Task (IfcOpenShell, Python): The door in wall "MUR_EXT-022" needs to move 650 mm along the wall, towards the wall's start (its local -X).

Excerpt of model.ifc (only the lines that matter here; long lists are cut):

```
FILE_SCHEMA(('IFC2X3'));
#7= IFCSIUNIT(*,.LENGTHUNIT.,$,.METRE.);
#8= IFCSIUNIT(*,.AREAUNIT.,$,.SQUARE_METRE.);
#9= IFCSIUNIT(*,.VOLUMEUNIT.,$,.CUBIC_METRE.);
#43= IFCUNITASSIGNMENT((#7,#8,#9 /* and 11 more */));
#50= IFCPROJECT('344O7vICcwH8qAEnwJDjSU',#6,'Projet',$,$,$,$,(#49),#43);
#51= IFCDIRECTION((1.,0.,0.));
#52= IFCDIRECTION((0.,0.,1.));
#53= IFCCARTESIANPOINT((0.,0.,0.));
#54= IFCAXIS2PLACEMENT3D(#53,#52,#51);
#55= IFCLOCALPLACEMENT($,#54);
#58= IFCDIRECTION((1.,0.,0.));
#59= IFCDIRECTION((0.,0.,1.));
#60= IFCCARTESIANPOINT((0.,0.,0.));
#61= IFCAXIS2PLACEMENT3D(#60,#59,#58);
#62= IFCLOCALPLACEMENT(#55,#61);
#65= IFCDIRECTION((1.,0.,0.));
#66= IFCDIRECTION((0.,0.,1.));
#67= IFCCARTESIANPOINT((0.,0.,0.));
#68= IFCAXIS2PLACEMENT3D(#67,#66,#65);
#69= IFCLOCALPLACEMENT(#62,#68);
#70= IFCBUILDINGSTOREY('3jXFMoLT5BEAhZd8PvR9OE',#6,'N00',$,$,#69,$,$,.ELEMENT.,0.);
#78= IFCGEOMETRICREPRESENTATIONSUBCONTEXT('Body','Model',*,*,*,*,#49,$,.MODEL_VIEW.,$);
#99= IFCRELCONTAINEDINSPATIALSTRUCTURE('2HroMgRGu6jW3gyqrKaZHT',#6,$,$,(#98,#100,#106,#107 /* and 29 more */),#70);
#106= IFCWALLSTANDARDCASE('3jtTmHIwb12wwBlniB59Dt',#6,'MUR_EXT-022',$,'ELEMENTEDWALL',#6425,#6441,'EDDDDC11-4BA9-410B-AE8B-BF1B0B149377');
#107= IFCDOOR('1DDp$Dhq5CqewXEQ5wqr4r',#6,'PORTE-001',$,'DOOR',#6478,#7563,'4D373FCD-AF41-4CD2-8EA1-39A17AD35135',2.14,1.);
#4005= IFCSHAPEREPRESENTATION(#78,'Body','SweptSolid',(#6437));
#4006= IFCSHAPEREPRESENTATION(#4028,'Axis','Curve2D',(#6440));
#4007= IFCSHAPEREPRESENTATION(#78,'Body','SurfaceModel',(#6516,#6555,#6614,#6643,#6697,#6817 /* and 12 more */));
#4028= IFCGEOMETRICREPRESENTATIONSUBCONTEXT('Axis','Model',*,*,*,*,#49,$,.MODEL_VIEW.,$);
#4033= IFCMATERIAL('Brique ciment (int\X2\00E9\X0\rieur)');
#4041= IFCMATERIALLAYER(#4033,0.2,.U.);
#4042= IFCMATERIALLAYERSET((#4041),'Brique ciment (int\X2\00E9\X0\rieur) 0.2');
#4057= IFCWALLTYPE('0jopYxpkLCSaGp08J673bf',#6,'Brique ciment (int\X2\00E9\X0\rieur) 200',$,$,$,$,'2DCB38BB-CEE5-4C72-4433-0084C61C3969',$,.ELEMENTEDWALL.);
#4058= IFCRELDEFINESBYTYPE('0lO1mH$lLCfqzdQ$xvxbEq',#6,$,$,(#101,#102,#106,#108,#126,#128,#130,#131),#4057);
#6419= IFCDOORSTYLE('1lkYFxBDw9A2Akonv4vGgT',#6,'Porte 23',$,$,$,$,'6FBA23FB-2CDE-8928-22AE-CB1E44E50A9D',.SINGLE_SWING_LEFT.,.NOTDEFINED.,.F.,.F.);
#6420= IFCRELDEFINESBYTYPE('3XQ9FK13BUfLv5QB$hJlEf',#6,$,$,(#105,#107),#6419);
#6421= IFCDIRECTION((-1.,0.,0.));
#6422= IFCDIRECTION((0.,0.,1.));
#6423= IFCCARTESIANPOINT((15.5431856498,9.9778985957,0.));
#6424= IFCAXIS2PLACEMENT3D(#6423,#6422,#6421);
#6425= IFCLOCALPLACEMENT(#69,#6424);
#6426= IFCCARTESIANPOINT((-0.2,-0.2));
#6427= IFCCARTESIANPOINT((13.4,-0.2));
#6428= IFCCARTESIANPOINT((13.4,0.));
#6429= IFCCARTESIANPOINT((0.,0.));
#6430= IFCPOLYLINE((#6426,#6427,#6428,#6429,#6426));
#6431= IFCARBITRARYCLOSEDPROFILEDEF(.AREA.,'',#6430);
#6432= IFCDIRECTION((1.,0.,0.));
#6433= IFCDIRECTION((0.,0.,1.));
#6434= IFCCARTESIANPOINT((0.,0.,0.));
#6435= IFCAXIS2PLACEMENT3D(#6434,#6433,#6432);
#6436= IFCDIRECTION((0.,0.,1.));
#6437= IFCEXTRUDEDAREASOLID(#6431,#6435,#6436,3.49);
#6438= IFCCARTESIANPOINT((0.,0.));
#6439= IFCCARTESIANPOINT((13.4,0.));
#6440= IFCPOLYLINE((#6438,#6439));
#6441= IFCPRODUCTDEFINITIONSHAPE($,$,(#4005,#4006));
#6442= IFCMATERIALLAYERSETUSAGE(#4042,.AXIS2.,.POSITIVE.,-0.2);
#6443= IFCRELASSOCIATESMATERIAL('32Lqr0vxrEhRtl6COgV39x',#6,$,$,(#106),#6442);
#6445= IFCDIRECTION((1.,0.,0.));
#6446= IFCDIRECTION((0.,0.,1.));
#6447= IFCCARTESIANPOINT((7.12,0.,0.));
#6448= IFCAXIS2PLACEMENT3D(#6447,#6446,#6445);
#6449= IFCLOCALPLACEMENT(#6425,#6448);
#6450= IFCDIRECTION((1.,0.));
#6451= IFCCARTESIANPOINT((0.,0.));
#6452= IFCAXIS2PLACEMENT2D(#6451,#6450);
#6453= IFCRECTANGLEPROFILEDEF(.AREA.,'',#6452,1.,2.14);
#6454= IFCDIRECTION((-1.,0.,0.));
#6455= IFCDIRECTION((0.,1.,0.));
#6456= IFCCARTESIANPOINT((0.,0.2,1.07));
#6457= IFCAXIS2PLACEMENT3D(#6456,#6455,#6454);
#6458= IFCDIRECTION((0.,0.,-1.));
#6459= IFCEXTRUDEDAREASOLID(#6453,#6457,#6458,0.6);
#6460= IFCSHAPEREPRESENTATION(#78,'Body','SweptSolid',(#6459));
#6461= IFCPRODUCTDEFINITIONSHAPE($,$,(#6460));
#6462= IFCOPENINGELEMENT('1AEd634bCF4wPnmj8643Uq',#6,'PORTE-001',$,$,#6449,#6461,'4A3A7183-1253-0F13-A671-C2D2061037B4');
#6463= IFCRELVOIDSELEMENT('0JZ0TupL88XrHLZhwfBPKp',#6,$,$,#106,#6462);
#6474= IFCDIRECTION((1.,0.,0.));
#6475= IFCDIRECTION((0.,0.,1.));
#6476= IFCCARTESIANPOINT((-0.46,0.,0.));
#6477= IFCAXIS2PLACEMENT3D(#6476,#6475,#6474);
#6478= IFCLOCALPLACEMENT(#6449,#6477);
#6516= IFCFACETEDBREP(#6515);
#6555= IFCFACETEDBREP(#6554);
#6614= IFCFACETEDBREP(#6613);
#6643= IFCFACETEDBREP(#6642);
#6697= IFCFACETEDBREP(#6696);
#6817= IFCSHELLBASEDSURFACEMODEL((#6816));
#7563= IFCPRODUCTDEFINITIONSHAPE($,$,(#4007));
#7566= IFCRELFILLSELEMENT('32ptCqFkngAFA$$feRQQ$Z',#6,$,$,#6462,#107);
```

```python
import ifcopenshell
import ifcopenshell.api.geometry
import ifcopenshell.util.placement
import ifcopenshell.util.unit

model = ifcopenshell.open("model.ifc")
unit_scale = ifcopenshell.util.unit.calculate_unit_scale(model)

door = model.by_id(107)
opening = door.FillsVoids[0].RelatingOpeningElement
wall = opening.VoidsElements[0].RelatingBuildingElement

wall_matrix = ifcopenshell.util.placement.get_local_placement(wall.ObjectPlacement)
shift = wall_matrix[:3, 0] * -0.65 / unit_scale
before = ifcopenshell.util.placement.get_local_placement(door.ObjectPlacement)[:3, 3].copy()

# The door is placed relative to its opening, so it follows when the opening moves.
matrix = ifcopenshell.util.placement.get_local_placement(opening.ObjectPlacement)
matrix[:3, 3] += shift
ifcopenshell.api.geometry.edit_object_placement(
    model, product=opening, matrix=matrix, is_si=False, should_transform_children=True
)

after = ifcopenshell.util.placement.get_local_placement(door.ObjectPlacement)[:3, 3]
print("door moved by", (after - before).round(3) + 0.0)

model.write("model_updated.ifc")
```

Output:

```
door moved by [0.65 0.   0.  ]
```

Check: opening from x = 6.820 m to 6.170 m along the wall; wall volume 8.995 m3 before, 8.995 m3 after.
